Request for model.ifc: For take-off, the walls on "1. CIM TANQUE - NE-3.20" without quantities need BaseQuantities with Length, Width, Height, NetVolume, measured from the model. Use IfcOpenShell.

First a look at what the model holds.

```python
import ifcopenshell
import ifcopenshell.util.element
import ifcopenshell.util.unit

model = ifcopenshell.open("model.ifc")
print(model.schema)
for unit_type in ("LENGTHUNIT", "AREAUNIT", "VOLUMEUNIT"):
    print(unit_type, ifcopenshell.util.unit.calculate_unit_scale(model, unit_type))
storey = next(s for s in model.by_type("IfcBuildingStorey") if s.Name == "1. CIM TANQUE - NE-3.20")
walls = [e for e in ifcopenshell.util.element.get_decomposition(storey) if e.is_a("IfcWall")]
for e in sorted(walls, key=lambda e: e.id()):
    print(e.id(), e.is_a(), e.Name, list(ifcopenshell.util.element.get_psets(e, qtos_only=True)), sep=" | ")
```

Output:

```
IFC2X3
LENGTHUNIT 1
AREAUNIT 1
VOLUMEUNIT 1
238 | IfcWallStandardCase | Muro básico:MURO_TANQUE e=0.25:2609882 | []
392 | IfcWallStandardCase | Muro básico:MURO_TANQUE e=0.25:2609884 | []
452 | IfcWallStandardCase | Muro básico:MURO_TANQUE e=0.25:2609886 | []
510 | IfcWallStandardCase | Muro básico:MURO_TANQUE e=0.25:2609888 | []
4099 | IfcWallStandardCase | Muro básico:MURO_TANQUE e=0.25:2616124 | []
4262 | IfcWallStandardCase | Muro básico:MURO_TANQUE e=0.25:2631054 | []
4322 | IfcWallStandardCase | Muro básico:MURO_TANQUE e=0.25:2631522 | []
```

```python
import ifcopenshell
import ifcopenshell.api.pset
import ifcopenshell.geom
import ifcopenshell.util.element
import ifcopenshell.util.shape
import ifcopenshell.util.unit

model = ifcopenshell.open("model.ifc")
unit_scale = ifcopenshell.util.unit.calculate_unit_scale(model)
volume_scale = ifcopenshell.util.unit.calculate_unit_scale(model, "VOLUMEUNIT")
settings = ifcopenshell.geom.settings()

storey = next(s for s in model.by_type("IfcBuildingStorey") if s.Name == "1. CIM TANQUE - NE-3.20")
walls = [e for e in ifcopenshell.util.element.get_decomposition(storey) if e.is_a("IfcWall")]

for e in sorted(walls, key=lambda e: e.id()):
    if ifcopenshell.util.element.get_psets(e, qtos_only=True, should_inherit=False):
        continue
    # Geometry comes back in metres, in the element's own axes.
    shape = ifcopenshell.geom.create_shape(settings, e)
    values = {
        "Length": ifcopenshell.util.shape.get_x(shape.geometry) / unit_scale,
        "Width": ifcopenshell.util.shape.get_y(shape.geometry) / unit_scale,
        "Height": ifcopenshell.util.shape.get_z(shape.geometry) / unit_scale,
        "NetVolume": ifcopenshell.util.shape.get_volume(shape.geometry) / volume_scale,
    }
    qto = ifcopenshell.api.pset.add_qto(model, product=e, name="BaseQuantities")
    ifcopenshell.api.pset.edit_qto(model, qto=qto, properties=values)
    print(e.id(), {k: round(v, 3) for k, v in values.items()})

model.write("model_updated.ifc")
```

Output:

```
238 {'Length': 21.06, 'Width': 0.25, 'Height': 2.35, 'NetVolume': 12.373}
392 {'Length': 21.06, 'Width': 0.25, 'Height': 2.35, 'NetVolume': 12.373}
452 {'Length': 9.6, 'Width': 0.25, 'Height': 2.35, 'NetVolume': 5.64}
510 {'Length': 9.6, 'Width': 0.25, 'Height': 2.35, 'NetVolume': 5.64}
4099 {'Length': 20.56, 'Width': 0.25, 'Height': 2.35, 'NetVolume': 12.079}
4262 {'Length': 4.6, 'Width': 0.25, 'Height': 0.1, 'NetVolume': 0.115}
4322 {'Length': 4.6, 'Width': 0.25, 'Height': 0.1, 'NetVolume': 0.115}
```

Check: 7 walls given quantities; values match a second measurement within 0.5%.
